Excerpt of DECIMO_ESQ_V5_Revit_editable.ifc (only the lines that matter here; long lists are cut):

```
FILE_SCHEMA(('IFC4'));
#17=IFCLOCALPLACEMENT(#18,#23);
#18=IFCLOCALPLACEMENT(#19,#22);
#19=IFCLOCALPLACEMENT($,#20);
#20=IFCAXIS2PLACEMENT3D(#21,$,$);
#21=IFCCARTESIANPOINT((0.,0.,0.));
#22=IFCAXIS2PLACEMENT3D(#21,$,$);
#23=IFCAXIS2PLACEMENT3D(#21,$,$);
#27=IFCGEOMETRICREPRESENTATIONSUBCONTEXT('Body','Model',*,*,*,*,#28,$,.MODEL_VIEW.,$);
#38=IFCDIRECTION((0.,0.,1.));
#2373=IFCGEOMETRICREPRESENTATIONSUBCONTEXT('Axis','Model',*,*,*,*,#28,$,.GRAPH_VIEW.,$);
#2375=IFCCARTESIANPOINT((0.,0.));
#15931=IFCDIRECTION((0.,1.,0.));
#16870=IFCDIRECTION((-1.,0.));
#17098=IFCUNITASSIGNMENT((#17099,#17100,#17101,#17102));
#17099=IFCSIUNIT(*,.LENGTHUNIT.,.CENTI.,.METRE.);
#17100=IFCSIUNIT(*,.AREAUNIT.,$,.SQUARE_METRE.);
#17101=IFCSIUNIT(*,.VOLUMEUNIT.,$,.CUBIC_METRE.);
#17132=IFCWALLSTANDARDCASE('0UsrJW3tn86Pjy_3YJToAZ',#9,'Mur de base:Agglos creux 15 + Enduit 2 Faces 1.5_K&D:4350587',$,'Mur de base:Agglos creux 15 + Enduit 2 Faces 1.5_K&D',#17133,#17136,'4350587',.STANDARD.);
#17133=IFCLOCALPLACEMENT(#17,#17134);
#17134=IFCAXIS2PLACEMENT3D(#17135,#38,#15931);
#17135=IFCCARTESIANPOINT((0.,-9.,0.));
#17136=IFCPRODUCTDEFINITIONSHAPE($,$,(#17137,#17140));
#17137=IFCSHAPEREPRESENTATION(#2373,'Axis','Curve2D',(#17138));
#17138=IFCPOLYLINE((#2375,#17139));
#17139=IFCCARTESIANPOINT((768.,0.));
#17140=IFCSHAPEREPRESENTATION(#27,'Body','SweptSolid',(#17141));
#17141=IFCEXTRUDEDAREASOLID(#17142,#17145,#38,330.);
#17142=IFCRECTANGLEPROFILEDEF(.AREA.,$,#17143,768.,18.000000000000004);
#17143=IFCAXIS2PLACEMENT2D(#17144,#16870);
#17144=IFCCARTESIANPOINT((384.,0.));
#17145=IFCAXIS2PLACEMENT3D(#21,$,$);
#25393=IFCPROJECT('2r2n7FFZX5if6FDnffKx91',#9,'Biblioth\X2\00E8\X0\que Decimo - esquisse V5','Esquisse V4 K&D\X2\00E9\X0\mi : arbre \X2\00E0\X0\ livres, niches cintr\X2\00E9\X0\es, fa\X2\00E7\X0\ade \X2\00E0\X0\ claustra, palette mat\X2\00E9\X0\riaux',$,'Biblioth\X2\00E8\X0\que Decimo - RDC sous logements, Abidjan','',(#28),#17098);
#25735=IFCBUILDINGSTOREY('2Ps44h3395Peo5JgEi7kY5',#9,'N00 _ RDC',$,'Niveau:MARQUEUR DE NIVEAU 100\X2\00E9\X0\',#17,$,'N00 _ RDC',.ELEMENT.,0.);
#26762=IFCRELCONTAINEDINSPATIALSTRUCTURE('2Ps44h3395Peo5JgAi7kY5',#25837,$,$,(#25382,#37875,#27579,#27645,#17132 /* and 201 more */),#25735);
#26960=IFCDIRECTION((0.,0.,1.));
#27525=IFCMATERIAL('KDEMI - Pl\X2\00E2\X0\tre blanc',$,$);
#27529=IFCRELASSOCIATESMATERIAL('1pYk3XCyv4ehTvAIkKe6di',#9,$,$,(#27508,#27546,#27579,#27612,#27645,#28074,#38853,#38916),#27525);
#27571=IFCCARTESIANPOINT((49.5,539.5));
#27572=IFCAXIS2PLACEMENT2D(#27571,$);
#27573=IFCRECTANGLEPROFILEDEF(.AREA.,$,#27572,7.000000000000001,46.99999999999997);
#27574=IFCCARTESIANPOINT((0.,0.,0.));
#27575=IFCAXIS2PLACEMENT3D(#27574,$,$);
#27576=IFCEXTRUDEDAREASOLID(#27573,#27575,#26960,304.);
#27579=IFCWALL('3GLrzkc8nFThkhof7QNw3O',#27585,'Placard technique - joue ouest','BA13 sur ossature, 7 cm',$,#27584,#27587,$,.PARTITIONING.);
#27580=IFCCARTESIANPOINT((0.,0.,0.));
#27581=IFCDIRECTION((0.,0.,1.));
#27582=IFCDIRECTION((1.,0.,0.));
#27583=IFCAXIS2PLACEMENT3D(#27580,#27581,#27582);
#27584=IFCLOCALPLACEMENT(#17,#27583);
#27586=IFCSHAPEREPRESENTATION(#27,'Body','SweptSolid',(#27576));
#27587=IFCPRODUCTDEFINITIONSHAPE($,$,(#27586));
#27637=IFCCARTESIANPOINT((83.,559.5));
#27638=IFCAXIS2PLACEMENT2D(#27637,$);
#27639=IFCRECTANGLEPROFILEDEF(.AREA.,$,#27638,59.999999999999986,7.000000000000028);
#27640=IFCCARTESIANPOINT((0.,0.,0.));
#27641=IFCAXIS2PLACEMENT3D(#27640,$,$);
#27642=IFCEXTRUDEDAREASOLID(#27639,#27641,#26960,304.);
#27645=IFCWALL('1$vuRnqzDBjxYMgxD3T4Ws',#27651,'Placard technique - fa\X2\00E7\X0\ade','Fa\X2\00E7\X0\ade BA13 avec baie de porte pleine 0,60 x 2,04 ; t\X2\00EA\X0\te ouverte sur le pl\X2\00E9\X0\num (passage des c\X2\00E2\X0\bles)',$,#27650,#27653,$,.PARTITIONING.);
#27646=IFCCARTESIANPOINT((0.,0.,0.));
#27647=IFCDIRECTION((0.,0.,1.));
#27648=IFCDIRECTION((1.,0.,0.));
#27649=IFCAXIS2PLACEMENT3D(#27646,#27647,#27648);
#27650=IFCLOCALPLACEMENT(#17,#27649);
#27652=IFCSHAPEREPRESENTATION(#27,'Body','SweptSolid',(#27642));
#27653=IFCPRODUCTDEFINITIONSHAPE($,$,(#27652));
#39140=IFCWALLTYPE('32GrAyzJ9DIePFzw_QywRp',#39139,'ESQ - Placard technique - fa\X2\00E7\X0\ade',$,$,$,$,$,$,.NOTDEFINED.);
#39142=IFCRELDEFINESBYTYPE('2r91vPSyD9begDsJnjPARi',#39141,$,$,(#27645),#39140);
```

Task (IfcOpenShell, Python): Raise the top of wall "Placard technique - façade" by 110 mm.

```python
import ifcopenshell
import ifcopenshell.geom
import ifcopenshell.util.representation
import ifcopenshell.util.shape
import ifcopenshell.util.unit

model = ifcopenshell.open("DECIMO_ESQ_V5_Revit_editable.ifc")
unit_scale = ifcopenshell.util.unit.calculate_unit_scale(model)
settings = ifcopenshell.geom.settings()


def volume(element):
    """Net volume in cubic metres, openings subtracted."""
    shape = ifcopenshell.geom.create_shape(settings, element)
    return ifcopenshell.util.shape.get_volume(shape.geometry)


wall = model.by_guid("1$vuRnqzDBjxYMgxD3T4Ws")
before = volume(wall)

body = ifcopenshell.util.representation.get_representation(wall, "Model", "Body")
solid = body.Items[0]
old_height = solid.Depth
solid.Depth += 0.11 / unit_scale
after = volume(wall)

print(f"height {old_height:g} -> {solid.Depth:g}, volume {before:.3f} -> {after:.3f} m3")

model.write("DECIMO_ESQ_V5_Revit_editable_updated.ifc")
```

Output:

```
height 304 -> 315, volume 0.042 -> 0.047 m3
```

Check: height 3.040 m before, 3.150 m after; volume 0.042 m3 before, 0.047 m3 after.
